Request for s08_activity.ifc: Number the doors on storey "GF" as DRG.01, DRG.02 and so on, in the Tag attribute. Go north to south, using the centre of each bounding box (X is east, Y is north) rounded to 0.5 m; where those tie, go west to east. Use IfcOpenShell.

First a look at what the model holds.

```python
import ifcopenshell
import ifcopenshell.util.element
import ifcopenshell.util.placement

model = ifcopenshell.open("s08_activity.ifc")
print(model.schema)
storey = next(s for s in model.by_type("IfcBuildingStorey") if s.Name == "GF")
doors = [e for e in ifcopenshell.util.element.get_decomposition(storey) if e.is_a("IfcDoor")]
for e in sorted(doors, key=lambda e: e.id()):
    origin = ifcopenshell.util.placement.get_local_placement(e.ObjectPlacement)[:3, 3]
    print(e.id(), e.Tag, e.Name, origin.round(2) + 0.0, sep=" | ")
```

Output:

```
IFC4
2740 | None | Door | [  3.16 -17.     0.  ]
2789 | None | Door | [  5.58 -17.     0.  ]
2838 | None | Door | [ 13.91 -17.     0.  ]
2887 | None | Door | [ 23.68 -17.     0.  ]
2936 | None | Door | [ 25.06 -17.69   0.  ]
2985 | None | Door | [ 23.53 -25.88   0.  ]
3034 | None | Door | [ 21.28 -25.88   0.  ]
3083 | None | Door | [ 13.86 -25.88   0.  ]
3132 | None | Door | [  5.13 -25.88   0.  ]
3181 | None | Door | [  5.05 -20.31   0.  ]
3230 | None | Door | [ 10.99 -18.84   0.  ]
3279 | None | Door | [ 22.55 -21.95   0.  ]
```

```python
import ifcopenshell
import ifcopenshell.geom
import ifcopenshell.util.element
import ifcopenshell.util.shape

model = ifcopenshell.open("s08_activity.ifc")
settings = ifcopenshell.geom.settings()
settings.set("use-world-coords", True)


def centre(element):
    shape = ifcopenshell.geom.create_shape(settings, element)
    return ifcopenshell.util.shape.get_bbox_centroid(shape.geometry)


storey = next(s for s in model.by_type("IfcBuildingStorey") if s.Name == "GF")
doors = [e for e in ifcopenshell.util.element.get_decomposition(storey) if e.is_a("IfcDoor")]

# Insertion points can sit at a corner or the storey origin, so sort by the geometry (in metres).
centres = {e: centre(e) for e in doors}
doors.sort(key=lambda e: (-round(centres[e][1] / 0.5), centres[e][0]))

for i, e in enumerate(doors, start=1):
    number = f"DRG.{i:02d}"
    e.Tag = number
    print(e.id(), number)

model.write("s08_activity_v2.ifc")
```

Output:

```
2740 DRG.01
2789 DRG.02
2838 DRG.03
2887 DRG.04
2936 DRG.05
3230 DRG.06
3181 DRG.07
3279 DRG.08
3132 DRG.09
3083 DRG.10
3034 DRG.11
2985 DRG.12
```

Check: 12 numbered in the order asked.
